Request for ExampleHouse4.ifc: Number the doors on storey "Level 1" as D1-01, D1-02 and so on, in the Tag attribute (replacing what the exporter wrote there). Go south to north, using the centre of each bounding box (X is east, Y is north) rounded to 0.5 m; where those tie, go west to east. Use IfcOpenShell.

First a look at what the model holds.

```python
import ifcopenshell
import ifcopenshell.util.element
import ifcopenshell.util.placement

model = ifcopenshell.open("ExampleHouse4.ifc")
print(model.schema)
storey = next(s for s in model.by_type("IfcBuildingStorey") if s.Name == "Level 1")
doors = [e for e in ifcopenshell.util.element.get_decomposition(storey) if e.is_a("IfcDoor")]
for e in sorted(doors, key=lambda e: e.id()):
    origin = ifcopenshell.util.placement.get_local_placement(e.ObjectPlacement)[:3, 3]
    print(e.id(), e.Tag, e.Name, origin.round(2) + 0.0, sep=" | ")
```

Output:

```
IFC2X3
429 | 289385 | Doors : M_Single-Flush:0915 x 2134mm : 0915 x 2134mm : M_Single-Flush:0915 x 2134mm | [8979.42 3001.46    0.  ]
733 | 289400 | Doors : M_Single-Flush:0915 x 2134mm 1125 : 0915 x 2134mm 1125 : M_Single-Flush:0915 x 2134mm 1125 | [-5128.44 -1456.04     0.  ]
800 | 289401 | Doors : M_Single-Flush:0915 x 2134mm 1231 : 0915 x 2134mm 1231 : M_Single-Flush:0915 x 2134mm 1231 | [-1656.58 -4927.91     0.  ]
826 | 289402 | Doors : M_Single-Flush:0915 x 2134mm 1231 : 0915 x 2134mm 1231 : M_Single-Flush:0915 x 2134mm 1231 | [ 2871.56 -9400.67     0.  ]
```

```python
import ifcopenshell
import ifcopenshell.geom
import ifcopenshell.util.element
import ifcopenshell.util.shape

model = ifcopenshell.open("ExampleHouse4.ifc")
settings = ifcopenshell.geom.settings()
settings.set("use-world-coords", True)


def centre(element):
    shape = ifcopenshell.geom.create_shape(settings, element)
    return ifcopenshell.util.shape.get_bbox_centroid(shape.geometry)


storey = next(s for s in model.by_type("IfcBuildingStorey") if s.Name == "Level 1")
doors = [e for e in ifcopenshell.util.element.get_decomposition(storey) if e.is_a("IfcDoor")]

# Insertion points can sit at a corner or the storey origin, so sort by the geometry (in metres).
centres = {e: centre(e) for e in doors}
doors.sort(key=lambda e: (round(centres[e][1] / 0.5), centres[e][0]))

for i, e in enumerate(doors, start=1):
    number = f"D1-{i:02d}"
    e.Tag = number
    print(e.id(), number)

model.write("ExampleHouse4_updated.ifc")
```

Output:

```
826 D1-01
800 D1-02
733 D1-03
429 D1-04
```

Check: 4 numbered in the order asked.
